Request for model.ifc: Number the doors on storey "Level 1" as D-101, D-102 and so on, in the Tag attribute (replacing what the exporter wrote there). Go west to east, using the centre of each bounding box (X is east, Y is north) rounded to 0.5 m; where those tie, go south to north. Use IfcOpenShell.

First a look at what the model holds.

```python
import ifcopenshell
import ifcopenshell.util.element
import ifcopenshell.util.placement

model = ifcopenshell.open("model.ifc")
print(model.schema)
storey = next(s for s in model.by_type("IfcBuildingStorey") if s.Name == "Level 1")
doors = [e for e in ifcopenshell.util.element.get_decomposition(storey) if e.is_a("IfcDoor")]
for e in sorted(doors, key=lambda e: e.id()):
    origin = ifcopenshell.util.placement.get_local_placement(e.ObjectPlacement)[:3, 3]
    print(e.id(), e.Tag, e.Name, origin.round(2) + 0.0, sep=" | ")
```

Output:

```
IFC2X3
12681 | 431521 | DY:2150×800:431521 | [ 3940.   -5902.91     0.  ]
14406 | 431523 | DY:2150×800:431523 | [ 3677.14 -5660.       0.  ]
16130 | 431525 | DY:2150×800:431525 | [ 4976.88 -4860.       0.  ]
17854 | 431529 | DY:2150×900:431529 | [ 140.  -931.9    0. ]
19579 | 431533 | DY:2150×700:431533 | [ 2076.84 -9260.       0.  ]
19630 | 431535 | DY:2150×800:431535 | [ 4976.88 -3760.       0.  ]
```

```python
import ifcopenshell
import ifcopenshell.geom
import ifcopenshell.util.element
import ifcopenshell.util.shape

model = ifcopenshell.open("model.ifc")
settings = ifcopenshell.geom.settings()
settings.set("use-world-coords", True)


def centre(element):
    shape = ifcopenshell.geom.create_shape(settings, element)
    return ifcopenshell.util.shape.get_bbox_centroid(shape.geometry)


storey = next(s for s in model.by_type("IfcBuildingStorey") if s.Name == "Level 1")
doors = [e for e in ifcopenshell.util.element.get_decomposition(storey) if e.is_a("IfcDoor")]

# Insertion points can sit at a corner or the storey origin, so sort by the geometry (in metres).
centres = {e: centre(e) for e in doors}
doors.sort(key=lambda e: (round(centres[e][0] / 0.5), centres[e][1]))

for i, e in enumerate(doors, start=1):
    number = f"D-1{i:02d}"
    e.Tag = number
    print(e.id(), number)

model.write("model_v2.ifc")
```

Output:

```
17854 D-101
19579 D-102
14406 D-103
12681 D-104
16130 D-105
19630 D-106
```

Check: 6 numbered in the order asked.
